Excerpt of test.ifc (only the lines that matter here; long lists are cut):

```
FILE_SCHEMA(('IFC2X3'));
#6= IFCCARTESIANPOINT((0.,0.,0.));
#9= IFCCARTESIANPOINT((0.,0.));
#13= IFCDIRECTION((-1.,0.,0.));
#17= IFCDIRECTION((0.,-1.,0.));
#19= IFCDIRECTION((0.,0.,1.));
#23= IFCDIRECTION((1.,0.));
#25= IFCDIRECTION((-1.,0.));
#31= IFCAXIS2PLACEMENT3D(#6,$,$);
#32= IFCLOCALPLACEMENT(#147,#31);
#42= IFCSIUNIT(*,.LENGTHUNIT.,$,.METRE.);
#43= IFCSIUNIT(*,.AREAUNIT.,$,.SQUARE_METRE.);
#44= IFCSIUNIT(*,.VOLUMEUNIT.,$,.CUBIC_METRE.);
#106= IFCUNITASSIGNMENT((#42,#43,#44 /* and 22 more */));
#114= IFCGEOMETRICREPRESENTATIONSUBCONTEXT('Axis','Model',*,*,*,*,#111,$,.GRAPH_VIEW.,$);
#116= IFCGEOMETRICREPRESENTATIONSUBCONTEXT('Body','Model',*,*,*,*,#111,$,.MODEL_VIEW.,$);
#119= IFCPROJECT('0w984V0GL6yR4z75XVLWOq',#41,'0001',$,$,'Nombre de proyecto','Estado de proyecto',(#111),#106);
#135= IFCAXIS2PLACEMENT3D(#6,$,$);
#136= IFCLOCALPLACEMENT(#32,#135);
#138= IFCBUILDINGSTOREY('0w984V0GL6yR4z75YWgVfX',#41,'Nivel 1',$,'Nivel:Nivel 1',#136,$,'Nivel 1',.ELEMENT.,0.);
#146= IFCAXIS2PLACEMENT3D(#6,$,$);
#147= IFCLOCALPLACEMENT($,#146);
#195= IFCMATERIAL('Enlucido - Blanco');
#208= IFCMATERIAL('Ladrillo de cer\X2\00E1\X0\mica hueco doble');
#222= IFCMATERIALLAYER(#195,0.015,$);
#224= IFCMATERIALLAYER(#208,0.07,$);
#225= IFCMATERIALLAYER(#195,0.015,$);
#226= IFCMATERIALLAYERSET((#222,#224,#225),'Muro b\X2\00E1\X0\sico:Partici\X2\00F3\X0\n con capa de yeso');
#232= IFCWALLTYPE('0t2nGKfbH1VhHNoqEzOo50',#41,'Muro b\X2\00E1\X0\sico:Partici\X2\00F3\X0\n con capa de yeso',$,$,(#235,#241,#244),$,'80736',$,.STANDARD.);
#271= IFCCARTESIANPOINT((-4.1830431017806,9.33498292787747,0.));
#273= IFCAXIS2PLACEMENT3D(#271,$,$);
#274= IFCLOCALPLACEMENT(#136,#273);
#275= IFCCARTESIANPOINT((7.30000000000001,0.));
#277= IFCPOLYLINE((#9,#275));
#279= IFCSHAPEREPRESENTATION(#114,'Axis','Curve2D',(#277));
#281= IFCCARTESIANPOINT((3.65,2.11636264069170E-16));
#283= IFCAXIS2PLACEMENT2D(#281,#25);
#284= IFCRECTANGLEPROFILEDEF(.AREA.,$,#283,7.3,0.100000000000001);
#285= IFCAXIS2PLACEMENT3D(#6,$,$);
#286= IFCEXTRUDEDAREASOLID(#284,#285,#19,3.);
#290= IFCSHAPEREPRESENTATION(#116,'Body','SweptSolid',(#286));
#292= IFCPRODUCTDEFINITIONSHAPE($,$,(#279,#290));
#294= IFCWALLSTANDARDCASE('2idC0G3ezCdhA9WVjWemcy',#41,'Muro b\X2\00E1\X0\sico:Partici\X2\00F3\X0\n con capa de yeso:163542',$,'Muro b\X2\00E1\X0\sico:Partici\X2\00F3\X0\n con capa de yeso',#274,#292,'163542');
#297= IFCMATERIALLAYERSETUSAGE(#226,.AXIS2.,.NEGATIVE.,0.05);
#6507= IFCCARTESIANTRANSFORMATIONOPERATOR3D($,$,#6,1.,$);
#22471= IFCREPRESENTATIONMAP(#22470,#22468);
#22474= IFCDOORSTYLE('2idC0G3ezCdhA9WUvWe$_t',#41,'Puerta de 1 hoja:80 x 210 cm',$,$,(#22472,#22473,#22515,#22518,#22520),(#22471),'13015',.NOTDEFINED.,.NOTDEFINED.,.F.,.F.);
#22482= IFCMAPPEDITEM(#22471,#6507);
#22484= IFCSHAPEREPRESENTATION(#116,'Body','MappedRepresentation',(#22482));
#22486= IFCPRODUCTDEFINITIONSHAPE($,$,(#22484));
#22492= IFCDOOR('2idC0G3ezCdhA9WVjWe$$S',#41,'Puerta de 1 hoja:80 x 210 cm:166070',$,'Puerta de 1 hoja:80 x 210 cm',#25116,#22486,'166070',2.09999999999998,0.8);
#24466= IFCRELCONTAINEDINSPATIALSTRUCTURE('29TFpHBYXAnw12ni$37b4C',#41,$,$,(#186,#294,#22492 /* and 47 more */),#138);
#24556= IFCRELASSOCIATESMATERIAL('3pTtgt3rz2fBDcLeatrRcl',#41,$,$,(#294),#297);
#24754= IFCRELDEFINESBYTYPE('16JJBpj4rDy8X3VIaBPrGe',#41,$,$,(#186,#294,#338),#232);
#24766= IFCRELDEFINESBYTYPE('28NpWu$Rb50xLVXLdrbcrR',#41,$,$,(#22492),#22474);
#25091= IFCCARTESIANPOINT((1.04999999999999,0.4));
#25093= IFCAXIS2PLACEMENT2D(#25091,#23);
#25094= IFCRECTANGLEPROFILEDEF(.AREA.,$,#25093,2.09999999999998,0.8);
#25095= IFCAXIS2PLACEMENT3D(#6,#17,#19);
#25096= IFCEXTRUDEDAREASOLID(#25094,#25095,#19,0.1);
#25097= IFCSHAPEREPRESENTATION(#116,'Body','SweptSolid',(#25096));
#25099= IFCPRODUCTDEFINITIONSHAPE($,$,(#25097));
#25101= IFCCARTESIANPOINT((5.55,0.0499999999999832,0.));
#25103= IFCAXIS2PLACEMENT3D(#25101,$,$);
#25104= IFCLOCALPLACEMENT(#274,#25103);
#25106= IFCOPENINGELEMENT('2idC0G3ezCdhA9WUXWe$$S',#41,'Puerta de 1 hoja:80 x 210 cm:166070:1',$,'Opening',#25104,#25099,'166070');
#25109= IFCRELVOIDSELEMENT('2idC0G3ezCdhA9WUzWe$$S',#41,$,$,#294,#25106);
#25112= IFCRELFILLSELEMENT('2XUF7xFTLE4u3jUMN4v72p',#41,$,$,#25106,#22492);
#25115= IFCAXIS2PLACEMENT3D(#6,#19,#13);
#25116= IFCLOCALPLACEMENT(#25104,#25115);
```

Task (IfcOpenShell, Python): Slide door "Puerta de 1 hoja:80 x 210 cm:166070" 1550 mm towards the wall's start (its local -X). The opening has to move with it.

```python
import ifcopenshell
import ifcopenshell.api.geometry
import ifcopenshell.util.placement
import ifcopenshell.util.unit

model = ifcopenshell.open("test.ifc")
unit_scale = ifcopenshell.util.unit.calculate_unit_scale(model)

door = model.by_guid("2idC0G3ezCdhA9WVjWe$$S")
opening = door.FillsVoids[0].RelatingOpeningElement
wall = opening.VoidsElements[0].RelatingBuildingElement

wall_matrix = ifcopenshell.util.placement.get_local_placement(wall.ObjectPlacement)
shift = wall_matrix[:3, 0] * -1.55 / unit_scale
before = ifcopenshell.util.placement.get_local_placement(door.ObjectPlacement)[:3, 3].copy()

# The door is placed relative to its opening, so it follows when the opening moves.
matrix = ifcopenshell.util.placement.get_local_placement(opening.ObjectPlacement)
matrix[:3, 3] += shift
ifcopenshell.api.geometry.edit_object_placement(
    model, product=opening, matrix=matrix, is_si=False, should_transform_children=True
)

after = ifcopenshell.util.placement.get_local_placement(door.ObjectPlacement)[:3, 3]
print("door moved by", (after - before).round(3) + 0.0)

model.write("test_v2.ifc")
```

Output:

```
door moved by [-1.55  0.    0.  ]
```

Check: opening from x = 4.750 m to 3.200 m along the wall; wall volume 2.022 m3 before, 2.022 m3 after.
